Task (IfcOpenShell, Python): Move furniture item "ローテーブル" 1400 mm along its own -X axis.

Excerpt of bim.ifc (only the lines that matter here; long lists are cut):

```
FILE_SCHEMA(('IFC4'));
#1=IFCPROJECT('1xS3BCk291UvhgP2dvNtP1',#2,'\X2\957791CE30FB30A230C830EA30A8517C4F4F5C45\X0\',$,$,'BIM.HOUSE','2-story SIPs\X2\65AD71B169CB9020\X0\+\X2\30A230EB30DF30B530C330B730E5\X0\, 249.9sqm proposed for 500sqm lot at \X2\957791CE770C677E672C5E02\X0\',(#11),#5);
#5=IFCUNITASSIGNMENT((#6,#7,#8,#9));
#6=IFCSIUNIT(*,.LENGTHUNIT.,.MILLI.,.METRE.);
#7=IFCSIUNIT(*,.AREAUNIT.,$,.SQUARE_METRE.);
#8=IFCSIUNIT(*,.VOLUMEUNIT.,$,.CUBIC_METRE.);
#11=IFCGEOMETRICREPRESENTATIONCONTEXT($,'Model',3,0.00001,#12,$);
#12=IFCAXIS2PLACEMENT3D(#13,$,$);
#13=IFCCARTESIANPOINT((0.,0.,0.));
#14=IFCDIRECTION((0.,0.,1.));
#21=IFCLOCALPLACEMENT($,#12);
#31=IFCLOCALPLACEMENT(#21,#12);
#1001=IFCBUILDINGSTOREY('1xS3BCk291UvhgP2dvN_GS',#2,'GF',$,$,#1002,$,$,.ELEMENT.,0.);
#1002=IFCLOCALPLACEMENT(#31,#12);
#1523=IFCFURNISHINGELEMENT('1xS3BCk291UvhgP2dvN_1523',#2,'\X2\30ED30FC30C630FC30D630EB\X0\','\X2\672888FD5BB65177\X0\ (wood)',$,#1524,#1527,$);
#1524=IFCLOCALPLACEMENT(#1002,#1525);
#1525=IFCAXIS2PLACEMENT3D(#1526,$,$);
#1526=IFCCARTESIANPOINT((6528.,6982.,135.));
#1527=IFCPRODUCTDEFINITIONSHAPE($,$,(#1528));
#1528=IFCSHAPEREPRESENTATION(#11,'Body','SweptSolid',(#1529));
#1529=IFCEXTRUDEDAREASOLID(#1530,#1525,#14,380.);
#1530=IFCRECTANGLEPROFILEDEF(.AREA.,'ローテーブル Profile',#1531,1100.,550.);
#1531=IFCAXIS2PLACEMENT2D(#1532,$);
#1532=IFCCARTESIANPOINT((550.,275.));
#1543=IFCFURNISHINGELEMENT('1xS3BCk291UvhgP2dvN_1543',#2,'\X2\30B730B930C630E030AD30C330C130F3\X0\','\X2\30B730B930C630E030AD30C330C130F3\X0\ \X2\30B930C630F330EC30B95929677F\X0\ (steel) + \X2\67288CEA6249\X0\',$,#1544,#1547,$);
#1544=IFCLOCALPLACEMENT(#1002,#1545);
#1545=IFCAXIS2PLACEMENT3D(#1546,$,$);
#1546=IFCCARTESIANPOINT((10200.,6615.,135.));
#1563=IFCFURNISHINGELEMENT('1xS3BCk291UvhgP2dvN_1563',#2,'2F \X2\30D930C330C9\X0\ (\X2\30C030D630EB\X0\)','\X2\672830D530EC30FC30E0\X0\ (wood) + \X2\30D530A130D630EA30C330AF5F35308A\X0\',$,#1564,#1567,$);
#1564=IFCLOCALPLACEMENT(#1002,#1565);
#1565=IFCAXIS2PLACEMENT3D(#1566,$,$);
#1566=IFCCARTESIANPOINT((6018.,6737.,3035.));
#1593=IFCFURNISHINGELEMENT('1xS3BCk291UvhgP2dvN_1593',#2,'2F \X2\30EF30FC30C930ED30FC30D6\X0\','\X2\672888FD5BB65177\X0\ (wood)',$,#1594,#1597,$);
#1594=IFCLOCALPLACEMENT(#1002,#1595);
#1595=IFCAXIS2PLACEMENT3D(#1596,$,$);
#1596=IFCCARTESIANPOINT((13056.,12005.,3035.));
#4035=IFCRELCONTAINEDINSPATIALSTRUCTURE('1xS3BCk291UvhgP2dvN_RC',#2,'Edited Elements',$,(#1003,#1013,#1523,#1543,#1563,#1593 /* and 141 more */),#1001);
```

```python
import ifcopenshell
import ifcopenshell.api.geometry
import ifcopenshell.util.placement

model = ifcopenshell.open("bim.ifc")

item = model.by_guid("1xS3BCk291UvhgP2dvN_1523")
matrix = ifcopenshell.util.placement.get_local_placement(item.ObjectPlacement)
matrix[:3, 3] -= matrix[:3, 0] * 1400.0
ifcopenshell.api.geometry.edit_object_placement(model, product=item, matrix=matrix, is_si=False)

print(ifcopenshell.util.placement.get_local_placement(item.ObjectPlacement).round(3) + 0.0)

model.write("bim_edited.ifc")
```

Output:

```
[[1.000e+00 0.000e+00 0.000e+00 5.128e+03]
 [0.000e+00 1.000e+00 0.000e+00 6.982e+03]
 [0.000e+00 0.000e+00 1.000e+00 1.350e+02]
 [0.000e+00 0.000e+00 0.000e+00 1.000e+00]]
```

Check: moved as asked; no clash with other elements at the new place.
